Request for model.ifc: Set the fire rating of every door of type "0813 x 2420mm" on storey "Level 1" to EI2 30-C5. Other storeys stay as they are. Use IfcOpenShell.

First a look at what the model holds.

```python
import ifcopenshell
import ifcopenshell.util.element

model = ifcopenshell.open("model.ifc")
print(model.schema)
storey = next(s for s in model.by_type("IfcBuildingStorey") if s.Name == "Level 1")
doors = [e for e in ifcopenshell.util.element.get_decomposition(storey) if e.is_a("IfcDoor")]
seen = {}
for e in doors:
    element_type = ifcopenshell.util.element.get_type(e)
    key = (element_type.Name if element_type != e and element_type else None, ifcopenshell.util.element.get_pset(e, "Pset_DoorCommon", "FireRating"))
    seen[key] = seen.get(key, 0) + 1
for (name, value), count in sorted(seen.items(), key=str):
    print(count, "x", name, "|", value)
```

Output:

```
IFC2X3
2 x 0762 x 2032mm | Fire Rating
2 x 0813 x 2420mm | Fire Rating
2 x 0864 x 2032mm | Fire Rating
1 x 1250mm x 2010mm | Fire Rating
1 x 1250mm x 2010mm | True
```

```python
import ifcopenshell
import ifcopenshell.api.pset
import ifcopenshell.util.element

model = ifcopenshell.open("model.ifc")

storey = next(s for s in model.by_type("IfcBuildingStorey") if s.Name == "Level 1")
doors = [e for e in ifcopenshell.util.element.get_decomposition(storey) if e.is_a("IfcDoor")]

count = 0
for e in doors:
    element_type = ifcopenshell.util.element.get_type(e)
    if element_type in (None, e) or element_type.Name != "0813 x 2420mm":
        continue
    # add_pset returns the element's existing set when there is one.
    pset = ifcopenshell.api.pset.add_pset(model, product=e, name="Pset_DoorCommon")
    ifcopenshell.api.pset.edit_pset(model, pset=pset, properties={"FireRating": "EI2 30-C5"})
    count += 1

print(count, "doors updated")

model.write("model_v2.ifc")
```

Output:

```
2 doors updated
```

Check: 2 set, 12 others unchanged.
